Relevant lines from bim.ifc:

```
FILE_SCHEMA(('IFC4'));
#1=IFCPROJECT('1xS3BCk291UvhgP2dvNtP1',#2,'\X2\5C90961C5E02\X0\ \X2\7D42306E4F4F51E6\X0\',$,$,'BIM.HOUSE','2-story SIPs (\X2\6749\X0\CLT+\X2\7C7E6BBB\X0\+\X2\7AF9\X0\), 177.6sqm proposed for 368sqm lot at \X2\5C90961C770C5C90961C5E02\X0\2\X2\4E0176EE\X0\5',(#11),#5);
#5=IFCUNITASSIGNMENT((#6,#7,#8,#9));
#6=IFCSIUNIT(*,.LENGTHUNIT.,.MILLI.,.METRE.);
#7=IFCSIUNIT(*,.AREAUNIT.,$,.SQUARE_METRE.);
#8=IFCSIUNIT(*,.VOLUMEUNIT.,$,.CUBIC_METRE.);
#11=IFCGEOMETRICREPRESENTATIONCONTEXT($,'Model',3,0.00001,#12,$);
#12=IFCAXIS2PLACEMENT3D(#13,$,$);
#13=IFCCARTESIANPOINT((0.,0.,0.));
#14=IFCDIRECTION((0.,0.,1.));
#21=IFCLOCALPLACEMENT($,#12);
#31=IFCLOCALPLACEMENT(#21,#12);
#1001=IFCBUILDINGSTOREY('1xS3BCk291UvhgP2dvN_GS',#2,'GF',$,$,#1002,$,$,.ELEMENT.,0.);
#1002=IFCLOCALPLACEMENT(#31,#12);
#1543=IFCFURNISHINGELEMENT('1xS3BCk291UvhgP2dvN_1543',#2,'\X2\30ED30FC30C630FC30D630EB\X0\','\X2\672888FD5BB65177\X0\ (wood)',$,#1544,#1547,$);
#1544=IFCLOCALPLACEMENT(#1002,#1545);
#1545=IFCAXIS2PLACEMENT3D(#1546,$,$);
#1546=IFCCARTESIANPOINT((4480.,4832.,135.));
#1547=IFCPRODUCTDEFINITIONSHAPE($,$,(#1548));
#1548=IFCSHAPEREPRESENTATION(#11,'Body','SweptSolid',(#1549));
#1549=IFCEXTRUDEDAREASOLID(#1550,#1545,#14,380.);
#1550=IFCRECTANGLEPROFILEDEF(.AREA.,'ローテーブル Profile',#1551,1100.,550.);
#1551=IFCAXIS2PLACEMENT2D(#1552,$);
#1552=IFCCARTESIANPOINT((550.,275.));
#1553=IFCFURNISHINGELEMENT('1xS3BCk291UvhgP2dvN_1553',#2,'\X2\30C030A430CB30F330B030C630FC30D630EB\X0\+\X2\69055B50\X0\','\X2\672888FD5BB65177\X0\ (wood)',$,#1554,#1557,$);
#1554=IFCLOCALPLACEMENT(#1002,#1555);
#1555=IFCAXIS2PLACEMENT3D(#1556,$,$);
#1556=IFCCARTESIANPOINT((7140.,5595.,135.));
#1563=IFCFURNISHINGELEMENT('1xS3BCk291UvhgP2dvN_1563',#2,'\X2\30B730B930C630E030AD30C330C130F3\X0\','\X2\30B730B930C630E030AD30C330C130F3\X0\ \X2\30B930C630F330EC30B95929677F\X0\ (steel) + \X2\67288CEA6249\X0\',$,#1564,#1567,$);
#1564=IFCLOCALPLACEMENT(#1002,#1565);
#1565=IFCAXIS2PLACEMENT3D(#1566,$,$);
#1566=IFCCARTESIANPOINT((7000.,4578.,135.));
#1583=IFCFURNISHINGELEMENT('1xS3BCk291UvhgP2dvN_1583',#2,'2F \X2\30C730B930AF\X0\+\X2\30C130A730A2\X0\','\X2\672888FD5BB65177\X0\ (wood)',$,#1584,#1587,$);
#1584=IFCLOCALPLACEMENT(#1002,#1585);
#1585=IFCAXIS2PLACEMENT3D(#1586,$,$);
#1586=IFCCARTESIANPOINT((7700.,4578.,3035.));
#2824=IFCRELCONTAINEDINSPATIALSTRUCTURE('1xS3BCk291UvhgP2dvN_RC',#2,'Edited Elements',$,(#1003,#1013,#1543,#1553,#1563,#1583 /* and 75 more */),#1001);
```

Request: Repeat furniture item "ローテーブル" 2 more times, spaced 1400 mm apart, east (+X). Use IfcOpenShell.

```python
import numpy as np
import ifcopenshell
import ifcopenshell.api.geometry
import ifcopenshell.api.root
import ifcopenshell.util.element
import ifcopenshell.util.placement
import ifcopenshell.util.unit

model = ifcopenshell.open("bim.ifc")
unit_scale = ifcopenshell.util.unit.calculate_unit_scale(model)


def reuse_history(source, copy):
    """copy_class also copies each property set's owner history, people and application; keep the originals."""
    for rel in copy.IsDefinedBy:
        if rel.is_a("IfcRelDefinesByProperties") and (history := rel.RelatingPropertyDefinition.OwnerHistory):
            rel.RelatingPropertyDefinition.OwnerHistory = source.OwnerHistory
            ifcopenshell.util.element.remove_deep2(model, history)


source = model.by_guid("1xS3BCk291UvhgP2dvN_1543")
base = ifcopenshell.util.placement.get_local_placement(source.ObjectPlacement)
step = np.array([1.0, 0.0, 0.0]) * 1.4 / unit_scale

for i in range(1, 3):
    copy = ifcopenshell.api.root.copy_class(model, product=source)
    copy.Representation = ifcopenshell.util.element.copy_deep(
        model, source.Representation, exclude=["IfcGeometricRepresentationContext", "IfcRepresentationMap"]
    )
    reuse_history(source, copy)
    matrix = base.copy()
    matrix[:3, 3] += i * step
    print("added at", matrix[:3, 3].round(3) + 0.0)
    ifcopenshell.api.geometry.edit_object_placement(model, product=copy, matrix=matrix, is_si=False)

model.write("bim_v2.ifc")
```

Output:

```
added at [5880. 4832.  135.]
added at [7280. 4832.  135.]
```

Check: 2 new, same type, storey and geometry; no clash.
